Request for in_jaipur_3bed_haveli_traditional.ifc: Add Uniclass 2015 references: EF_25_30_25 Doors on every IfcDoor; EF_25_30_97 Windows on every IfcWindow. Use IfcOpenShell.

First a look at what the model holds.

```python
import ifcopenshell

model = ifcopenshell.open("in_jaipur_3bed_haveli_traditional.ifc")
print(model.schema)
print("classifications:", [c.Name for c in model.by_type("IfcClassification")])
for ifc_class in ("IfcDoor", "IfcRoof", "IfcStair", "IfcWall", "IfcWindow"):
    print(ifc_class, len(model.by_type(ifc_class)))
```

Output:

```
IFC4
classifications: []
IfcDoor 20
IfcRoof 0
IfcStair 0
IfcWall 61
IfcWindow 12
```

```python
import ifcopenshell
import ifcopenshell.api.classification

model = ifcopenshell.open("in_jaipur_3bed_haveli_traditional.ifc")

system = ifcopenshell.api.classification.add_classification(model, classification="Uniclass 2015")

codes = {
    "IfcDoor": ("EF_25_30_25", "Doors"),
    "IfcWindow": ("EF_25_30_97", "Windows"),
}
for ifc_class, (code, name) in codes.items():
    products = model.by_type(ifc_class)
    ifcopenshell.api.classification.add_reference(
        model, products=products, classification=system, identification=code, name=name
    )
    print(code, len(products))

model.write("in_jaipur_3bed_haveli_traditional_updated.ifc")
```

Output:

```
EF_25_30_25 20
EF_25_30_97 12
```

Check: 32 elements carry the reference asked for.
